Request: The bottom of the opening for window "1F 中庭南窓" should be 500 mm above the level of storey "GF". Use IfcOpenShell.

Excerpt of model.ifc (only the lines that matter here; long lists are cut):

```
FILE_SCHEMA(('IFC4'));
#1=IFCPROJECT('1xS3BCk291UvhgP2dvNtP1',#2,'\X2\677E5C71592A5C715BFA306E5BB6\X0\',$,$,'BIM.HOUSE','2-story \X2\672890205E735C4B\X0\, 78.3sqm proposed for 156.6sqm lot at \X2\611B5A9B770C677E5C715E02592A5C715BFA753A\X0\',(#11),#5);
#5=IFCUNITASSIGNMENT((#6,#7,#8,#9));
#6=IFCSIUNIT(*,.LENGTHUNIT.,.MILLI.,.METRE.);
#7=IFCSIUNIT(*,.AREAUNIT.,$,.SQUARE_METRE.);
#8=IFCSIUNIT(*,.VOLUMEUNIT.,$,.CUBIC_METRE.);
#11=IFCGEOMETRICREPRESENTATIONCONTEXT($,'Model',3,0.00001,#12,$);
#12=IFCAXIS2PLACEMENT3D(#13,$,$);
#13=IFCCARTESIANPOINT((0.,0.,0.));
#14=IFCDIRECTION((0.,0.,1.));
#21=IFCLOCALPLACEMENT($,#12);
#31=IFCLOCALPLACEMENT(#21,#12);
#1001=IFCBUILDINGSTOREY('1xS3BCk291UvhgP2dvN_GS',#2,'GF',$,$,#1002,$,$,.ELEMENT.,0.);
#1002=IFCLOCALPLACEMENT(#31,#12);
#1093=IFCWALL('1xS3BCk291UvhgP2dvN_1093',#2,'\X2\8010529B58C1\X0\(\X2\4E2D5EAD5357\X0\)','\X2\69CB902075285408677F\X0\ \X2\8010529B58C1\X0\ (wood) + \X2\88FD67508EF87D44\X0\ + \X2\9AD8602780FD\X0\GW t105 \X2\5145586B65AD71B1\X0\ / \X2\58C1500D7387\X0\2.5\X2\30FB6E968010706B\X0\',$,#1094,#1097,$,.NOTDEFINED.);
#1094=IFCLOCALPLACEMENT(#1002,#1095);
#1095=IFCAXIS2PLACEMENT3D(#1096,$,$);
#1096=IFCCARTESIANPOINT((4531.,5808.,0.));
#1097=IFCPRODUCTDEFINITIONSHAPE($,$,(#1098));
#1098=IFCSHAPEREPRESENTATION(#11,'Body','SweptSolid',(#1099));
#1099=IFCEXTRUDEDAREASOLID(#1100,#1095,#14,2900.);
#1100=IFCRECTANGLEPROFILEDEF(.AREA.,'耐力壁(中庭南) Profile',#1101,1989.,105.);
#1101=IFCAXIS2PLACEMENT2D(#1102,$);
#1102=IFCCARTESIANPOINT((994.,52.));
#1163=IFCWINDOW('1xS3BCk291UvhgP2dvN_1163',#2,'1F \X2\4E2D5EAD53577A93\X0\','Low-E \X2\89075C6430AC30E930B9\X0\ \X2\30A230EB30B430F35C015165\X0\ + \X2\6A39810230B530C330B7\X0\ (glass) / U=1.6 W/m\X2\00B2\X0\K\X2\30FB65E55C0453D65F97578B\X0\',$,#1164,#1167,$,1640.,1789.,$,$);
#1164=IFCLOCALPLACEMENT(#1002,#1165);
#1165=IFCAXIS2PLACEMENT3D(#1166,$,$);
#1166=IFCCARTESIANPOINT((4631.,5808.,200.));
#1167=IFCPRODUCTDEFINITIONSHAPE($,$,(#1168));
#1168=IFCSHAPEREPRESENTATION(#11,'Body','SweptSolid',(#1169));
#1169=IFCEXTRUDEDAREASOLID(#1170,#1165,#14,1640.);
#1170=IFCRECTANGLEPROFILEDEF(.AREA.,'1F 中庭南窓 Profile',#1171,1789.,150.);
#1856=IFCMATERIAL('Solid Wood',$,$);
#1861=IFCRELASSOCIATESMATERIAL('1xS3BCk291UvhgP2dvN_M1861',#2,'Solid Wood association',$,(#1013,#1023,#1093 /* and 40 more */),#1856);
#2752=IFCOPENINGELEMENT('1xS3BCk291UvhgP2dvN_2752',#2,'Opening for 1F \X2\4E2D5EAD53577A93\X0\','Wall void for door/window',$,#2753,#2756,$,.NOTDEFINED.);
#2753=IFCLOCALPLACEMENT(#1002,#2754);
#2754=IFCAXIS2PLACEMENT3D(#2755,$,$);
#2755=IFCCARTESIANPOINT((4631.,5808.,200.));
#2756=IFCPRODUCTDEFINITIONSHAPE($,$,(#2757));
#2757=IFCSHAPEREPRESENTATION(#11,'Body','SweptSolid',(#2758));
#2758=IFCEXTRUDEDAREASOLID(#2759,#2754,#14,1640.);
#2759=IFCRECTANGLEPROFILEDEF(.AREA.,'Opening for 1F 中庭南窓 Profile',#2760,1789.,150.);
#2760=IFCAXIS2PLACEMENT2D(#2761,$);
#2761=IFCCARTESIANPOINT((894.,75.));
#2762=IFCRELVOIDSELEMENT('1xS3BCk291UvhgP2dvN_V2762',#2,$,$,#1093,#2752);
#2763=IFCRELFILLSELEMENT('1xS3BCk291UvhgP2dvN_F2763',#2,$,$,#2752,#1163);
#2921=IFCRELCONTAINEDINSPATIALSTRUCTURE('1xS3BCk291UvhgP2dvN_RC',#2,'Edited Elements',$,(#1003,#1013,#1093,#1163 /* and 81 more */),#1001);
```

```python
import numpy as np
import ifcopenshell
import ifcopenshell.api.geometry
import ifcopenshell.geom
import ifcopenshell.util.element
import ifcopenshell.util.placement
import ifcopenshell.util.shape
import ifcopenshell.util.unit

model = ifcopenshell.open("model.ifc")
unit_scale = ifcopenshell.util.unit.calculate_unit_scale(model)

window = model.by_guid("1xS3BCk291UvhgP2dvN_1163")
opening = window.FillsVoids[0].RelatingOpeningElement
storey = ifcopenshell.util.element.get_container(window, ifc_class="IfcBuildingStorey")
level = ifcopenshell.util.placement.get_local_placement(storey.ObjectPlacement)[2, 3]

# The opening's origin need not be at the sill, so measure its lowest point.
shape = ifcopenshell.geom.create_shape(ifcopenshell.geom.settings(), opening)
bottom = ifcopenshell.util.shape.get_shape_bottom_elevation(shape, shape.geometry) / unit_scale
dz = level + 500.0 - bottom

shift = np.array([0.0, 0.0, dz])
# The window is not placed relative to its opening, so move both.
for product in (opening, window):
    matrix = ifcopenshell.util.placement.get_local_placement(product.ObjectPlacement)
    matrix[:3, 3] += shift
    ifcopenshell.api.geometry.edit_object_placement(model, product=product, matrix=matrix, is_si=False)

print(f"moved by {dz * unit_scale:+.3f} m")

model.write("model-out.ifc")
```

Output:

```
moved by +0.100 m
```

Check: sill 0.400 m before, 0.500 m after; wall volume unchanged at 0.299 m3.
